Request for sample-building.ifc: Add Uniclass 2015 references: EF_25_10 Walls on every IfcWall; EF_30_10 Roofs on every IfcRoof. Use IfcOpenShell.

First a look at what the model holds.

```python
import ifcopenshell

model = ifcopenshell.open("sample-building.ifc")
print(model.schema)
print("classifications:", [c.Name for c in model.by_type("IfcClassification")])
for ifc_class in ("IfcDoor", "IfcRoof", "IfcStair", "IfcWall", "IfcWindow"):
    print(ifc_class, len(model.by_type(ifc_class)))
```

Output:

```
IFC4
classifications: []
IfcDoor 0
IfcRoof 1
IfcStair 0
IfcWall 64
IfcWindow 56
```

```python
import ifcopenshell
import ifcopenshell.api.classification

model = ifcopenshell.open("sample-building.ifc")

system = ifcopenshell.api.classification.add_classification(model, classification="Uniclass 2015")

codes = {
    "IfcWall": ("EF_25_10", "Walls"),
    "IfcRoof": ("EF_30_10", "Roofs"),
}
for ifc_class, (code, name) in codes.items():
    products = model.by_type(ifc_class)
    ifcopenshell.api.classification.add_reference(
        model, products=products, classification=system, identification=code, name=name
    )
    print(code, len(products))

model.write("sample-building_v2.ifc")
```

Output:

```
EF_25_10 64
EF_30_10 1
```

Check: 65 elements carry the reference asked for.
